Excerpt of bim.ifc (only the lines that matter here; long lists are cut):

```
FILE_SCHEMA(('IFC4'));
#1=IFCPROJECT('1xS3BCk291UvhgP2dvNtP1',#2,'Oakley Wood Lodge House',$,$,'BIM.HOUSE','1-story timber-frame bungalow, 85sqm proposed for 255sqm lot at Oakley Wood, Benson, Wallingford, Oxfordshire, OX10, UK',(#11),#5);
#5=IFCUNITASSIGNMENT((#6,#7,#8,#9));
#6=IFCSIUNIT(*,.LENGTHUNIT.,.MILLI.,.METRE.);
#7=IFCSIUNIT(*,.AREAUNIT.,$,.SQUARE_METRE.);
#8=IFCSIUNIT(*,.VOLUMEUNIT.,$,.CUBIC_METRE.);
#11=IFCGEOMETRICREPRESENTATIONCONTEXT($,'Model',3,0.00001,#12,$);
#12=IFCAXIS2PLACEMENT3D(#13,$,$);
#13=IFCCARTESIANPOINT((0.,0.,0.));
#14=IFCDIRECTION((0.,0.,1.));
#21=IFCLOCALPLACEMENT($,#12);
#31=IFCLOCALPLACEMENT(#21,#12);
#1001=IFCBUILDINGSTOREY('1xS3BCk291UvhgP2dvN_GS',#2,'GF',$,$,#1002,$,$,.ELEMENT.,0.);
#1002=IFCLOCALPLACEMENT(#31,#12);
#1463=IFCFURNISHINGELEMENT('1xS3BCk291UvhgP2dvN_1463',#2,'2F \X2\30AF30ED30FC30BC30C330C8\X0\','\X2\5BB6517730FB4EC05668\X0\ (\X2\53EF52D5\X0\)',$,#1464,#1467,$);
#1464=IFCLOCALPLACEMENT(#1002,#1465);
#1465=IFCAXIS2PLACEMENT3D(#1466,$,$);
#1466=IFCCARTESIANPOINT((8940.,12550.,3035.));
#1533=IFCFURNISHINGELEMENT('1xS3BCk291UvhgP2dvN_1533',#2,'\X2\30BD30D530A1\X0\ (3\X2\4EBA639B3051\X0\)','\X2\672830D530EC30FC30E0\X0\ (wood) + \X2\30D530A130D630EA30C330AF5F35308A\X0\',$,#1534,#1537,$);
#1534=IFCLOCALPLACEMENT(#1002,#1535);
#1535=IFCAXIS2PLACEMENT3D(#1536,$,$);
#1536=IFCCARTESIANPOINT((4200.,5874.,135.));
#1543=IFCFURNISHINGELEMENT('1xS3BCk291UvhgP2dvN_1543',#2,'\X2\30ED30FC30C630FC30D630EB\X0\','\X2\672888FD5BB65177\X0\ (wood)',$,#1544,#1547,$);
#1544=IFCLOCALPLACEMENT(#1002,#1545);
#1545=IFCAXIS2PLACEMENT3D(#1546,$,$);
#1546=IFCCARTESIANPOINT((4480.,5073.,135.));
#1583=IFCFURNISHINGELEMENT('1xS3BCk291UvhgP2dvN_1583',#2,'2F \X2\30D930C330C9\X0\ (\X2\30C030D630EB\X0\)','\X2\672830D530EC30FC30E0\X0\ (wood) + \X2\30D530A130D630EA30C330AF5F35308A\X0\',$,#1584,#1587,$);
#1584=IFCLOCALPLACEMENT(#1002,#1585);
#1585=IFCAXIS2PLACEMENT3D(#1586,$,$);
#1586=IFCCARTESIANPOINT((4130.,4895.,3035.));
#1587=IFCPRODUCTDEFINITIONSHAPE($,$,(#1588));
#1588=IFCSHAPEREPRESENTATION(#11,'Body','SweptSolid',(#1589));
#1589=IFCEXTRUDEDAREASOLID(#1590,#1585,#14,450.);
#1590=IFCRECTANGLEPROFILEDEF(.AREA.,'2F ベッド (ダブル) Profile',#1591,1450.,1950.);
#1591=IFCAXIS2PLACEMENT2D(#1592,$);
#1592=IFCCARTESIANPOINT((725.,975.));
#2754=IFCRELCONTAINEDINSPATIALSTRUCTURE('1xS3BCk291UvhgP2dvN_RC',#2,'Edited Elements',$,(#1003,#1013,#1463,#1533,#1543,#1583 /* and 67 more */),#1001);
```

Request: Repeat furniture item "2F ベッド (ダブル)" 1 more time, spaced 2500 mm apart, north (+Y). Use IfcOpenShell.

```python
import numpy as np
import ifcopenshell
import ifcopenshell.api.geometry
import ifcopenshell.api.root
import ifcopenshell.util.element
import ifcopenshell.util.placement

model = ifcopenshell.open("bim.ifc")


def reuse_history(source, copy):
    """copy_class also copies each property set's owner history, people and application; keep the originals."""
    for rel in copy.IsDefinedBy:
        if rel.is_a("IfcRelDefinesByProperties") and (history := rel.RelatingPropertyDefinition.OwnerHistory):
            rel.RelatingPropertyDefinition.OwnerHistory = source.OwnerHistory
            ifcopenshell.util.element.remove_deep2(model, history)


source = model.by_id(1583)
base = ifcopenshell.util.placement.get_local_placement(source.ObjectPlacement)
step = np.array([0.0, 1.0, 0.0]) * 2500.0

for i in range(1, 2):
    copy = ifcopenshell.api.root.copy_class(model, product=source)
    copy.Representation = ifcopenshell.util.element.copy_deep(
        model, source.Representation, exclude=["IfcGeometricRepresentationContext", "IfcRepresentationMap"]
    )
    reuse_history(source, copy)
    matrix = base.copy()
    matrix[:3, 3] += i * step
    print("added at", matrix[:3, 3].round(3) + 0.0)
    ifcopenshell.api.geometry.edit_object_placement(model, product=copy, matrix=matrix, is_si=False)

model.write("bim_rev.ifc")
```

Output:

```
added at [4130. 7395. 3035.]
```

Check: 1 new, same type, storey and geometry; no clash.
